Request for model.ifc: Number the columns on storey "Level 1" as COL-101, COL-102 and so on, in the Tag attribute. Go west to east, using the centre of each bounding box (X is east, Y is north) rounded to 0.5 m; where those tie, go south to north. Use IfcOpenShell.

First a look at what the model holds.

```python
import ifcopenshell
import ifcopenshell.util.element
import ifcopenshell.util.placement

model = ifcopenshell.open("model.ifc")
print(model.schema)
storey = next(s for s in model.by_type("IfcBuildingStorey") if s.Name == "Level 1")
columns = [e for e in ifcopenshell.util.element.get_decomposition(storey) if e.is_a("IfcColumn")]
for e in sorted(columns, key=lambda e: e.id()):
    origin = ifcopenshell.util.placement.get_local_placement(e.ObjectPlacement)[:3, 3]
    print(e.id(), e.Tag, e.Name, origin.round(2) + 0.0, sep=" | ")
```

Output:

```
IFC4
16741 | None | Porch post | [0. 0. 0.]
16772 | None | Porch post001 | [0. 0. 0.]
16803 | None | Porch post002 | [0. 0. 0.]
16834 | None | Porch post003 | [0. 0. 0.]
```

```python
import ifcopenshell
import ifcopenshell.geom
import ifcopenshell.util.element
import ifcopenshell.util.shape

model = ifcopenshell.open("model.ifc")
settings = ifcopenshell.geom.settings()
settings.set("use-world-coords", True)


def centre(element):
    shape = ifcopenshell.geom.create_shape(settings, element)
    return ifcopenshell.util.shape.get_bbox_centroid(shape.geometry)


storey = next(s for s in model.by_type("IfcBuildingStorey") if s.Name == "Level 1")
columns = [e for e in ifcopenshell.util.element.get_decomposition(storey) if e.is_a("IfcColumn")]

# Insertion points can sit at a corner or the storey origin, so sort by the geometry (in metres).
centres = {e: centre(e) for e in columns}
columns.sort(key=lambda e: (round(centres[e][0] / 0.5), centres[e][1]))

for i, e in enumerate(columns, start=1):
    number = f"COL-1{i:02d}"
    e.Tag = number
    print(e.id(), number)

model.write("model_edited.ifc")
```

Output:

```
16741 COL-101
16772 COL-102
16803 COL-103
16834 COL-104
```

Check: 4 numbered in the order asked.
